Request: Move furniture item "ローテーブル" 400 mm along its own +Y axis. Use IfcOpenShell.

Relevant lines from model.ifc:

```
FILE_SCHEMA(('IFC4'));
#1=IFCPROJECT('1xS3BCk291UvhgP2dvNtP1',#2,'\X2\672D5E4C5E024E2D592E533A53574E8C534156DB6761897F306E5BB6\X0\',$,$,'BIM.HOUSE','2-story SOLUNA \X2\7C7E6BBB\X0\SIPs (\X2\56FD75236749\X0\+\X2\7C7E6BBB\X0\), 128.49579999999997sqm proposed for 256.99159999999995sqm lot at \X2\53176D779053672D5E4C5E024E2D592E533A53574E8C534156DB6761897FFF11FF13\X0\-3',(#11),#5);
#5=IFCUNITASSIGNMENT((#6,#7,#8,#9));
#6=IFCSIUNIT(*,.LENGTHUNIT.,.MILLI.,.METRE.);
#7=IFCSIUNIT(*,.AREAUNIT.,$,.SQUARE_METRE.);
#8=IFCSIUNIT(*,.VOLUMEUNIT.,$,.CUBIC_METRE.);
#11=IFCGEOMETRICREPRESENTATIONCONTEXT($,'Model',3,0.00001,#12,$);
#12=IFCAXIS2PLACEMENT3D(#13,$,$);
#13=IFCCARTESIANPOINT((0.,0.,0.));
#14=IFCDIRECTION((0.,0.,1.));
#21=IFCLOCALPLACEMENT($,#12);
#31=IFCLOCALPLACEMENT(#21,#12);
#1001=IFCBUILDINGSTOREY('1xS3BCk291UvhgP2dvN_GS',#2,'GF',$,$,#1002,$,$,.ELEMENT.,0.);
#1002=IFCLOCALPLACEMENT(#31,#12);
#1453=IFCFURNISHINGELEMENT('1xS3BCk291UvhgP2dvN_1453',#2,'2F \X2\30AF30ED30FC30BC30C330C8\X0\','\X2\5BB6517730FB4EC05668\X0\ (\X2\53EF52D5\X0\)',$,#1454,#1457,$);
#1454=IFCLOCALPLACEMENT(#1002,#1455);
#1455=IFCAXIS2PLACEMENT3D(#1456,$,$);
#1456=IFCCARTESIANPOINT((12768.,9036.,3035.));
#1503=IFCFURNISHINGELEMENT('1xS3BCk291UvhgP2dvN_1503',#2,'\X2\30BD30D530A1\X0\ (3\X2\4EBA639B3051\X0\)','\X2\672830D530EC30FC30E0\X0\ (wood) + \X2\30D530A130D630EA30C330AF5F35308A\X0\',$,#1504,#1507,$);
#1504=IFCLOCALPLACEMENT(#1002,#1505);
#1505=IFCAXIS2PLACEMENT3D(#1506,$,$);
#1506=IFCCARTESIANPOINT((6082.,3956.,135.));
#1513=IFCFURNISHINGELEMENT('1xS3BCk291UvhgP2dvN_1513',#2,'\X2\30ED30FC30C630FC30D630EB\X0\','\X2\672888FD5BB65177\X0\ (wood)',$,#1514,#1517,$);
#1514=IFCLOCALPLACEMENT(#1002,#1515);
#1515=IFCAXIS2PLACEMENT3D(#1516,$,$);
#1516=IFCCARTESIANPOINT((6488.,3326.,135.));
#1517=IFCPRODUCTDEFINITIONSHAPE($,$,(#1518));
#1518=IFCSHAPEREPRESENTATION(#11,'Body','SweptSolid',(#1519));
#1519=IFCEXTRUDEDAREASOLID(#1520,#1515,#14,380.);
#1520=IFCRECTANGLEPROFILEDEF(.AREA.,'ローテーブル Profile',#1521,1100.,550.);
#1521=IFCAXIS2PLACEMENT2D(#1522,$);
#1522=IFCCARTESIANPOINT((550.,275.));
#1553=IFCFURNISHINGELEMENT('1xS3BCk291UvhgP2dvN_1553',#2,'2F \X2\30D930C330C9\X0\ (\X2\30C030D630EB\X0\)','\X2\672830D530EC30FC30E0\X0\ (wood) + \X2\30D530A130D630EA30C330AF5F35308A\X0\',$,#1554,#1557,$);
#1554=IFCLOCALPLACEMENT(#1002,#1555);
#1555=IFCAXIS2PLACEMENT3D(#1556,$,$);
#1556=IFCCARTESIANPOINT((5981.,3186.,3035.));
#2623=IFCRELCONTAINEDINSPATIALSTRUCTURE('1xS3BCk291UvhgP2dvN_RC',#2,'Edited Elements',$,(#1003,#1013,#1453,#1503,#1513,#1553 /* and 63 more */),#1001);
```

```python
import ifcopenshell
import ifcopenshell.api.geometry
import ifcopenshell.util.placement
import ifcopenshell.util.unit

model = ifcopenshell.open("model.ifc")
unit_scale = ifcopenshell.util.unit.calculate_unit_scale(model)

item = model.by_guid("1xS3BCk291UvhgP2dvN_1513")
matrix = ifcopenshell.util.placement.get_local_placement(item.ObjectPlacement)
matrix[:3, 3] += matrix[:3, 1] * 0.4 / unit_scale
ifcopenshell.api.geometry.edit_object_placement(model, product=item, matrix=matrix, is_si=False)

print(ifcopenshell.util.placement.get_local_placement(item.ObjectPlacement).round(3) + 0.0)

model.write("model-out.ifc")
```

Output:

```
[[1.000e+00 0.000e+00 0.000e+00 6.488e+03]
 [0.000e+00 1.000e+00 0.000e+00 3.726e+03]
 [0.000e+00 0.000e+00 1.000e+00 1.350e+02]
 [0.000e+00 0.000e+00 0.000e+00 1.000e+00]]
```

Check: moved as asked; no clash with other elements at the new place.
